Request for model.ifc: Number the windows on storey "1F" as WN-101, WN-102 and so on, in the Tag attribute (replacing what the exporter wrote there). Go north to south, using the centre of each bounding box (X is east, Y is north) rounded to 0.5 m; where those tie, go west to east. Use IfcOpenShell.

First a look at what the model holds.

```python
import ifcopenshell
import ifcopenshell.util.element
import ifcopenshell.util.placement

model = ifcopenshell.open("model.ifc")
print(model.schema)
storey = next(s for s in model.by_type("IfcBuildingStorey") if s.Name == "1F")
windows = [e for e in ifcopenshell.util.element.get_decomposition(storey) if e.is_a("IfcWindow")]
for e in sorted(windows, key=lambda e: e.id()):
    origin = ifcopenshell.util.placement.get_local_placement(e.ObjectPlacement)[:3, 3]
    print(e.id(), e.Tag, e.Name, origin.round(2) + 0.0, sep=" | ")
```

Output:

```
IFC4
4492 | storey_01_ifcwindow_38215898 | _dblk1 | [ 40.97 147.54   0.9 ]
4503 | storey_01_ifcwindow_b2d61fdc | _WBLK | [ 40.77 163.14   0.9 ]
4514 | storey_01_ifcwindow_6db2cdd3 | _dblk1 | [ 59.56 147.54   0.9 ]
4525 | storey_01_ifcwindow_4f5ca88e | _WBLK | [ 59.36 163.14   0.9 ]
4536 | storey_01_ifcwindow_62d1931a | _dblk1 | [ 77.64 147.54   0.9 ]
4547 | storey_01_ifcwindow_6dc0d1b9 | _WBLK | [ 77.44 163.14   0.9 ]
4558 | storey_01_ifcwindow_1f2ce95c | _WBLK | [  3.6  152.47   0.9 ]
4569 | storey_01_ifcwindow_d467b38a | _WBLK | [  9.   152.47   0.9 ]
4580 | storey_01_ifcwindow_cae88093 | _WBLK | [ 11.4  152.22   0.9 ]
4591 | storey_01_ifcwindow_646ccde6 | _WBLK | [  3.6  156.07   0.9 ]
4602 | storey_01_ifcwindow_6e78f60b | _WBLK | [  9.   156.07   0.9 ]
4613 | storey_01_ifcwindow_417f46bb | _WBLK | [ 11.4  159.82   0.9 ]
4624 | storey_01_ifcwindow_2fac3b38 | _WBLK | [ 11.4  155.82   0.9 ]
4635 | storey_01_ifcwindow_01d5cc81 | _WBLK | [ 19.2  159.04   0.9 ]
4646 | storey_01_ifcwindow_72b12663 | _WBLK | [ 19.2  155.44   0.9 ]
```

```python
import ifcopenshell
import ifcopenshell.geom
import ifcopenshell.util.element
import ifcopenshell.util.shape

model = ifcopenshell.open("model.ifc")
settings = ifcopenshell.geom.settings()
settings.set("use-world-coords", True)


def centre(element):
    shape = ifcopenshell.geom.create_shape(settings, element)
    return ifcopenshell.util.shape.get_bbox_centroid(shape.geometry)


storey = next(s for s in model.by_type("IfcBuildingStorey") if s.Name == "1F")
windows = [e for e in ifcopenshell.util.element.get_decomposition(storey) if e.is_a("IfcWindow")]

# Insertion points can sit at a corner or the storey origin, so sort by the geometry (in metres).
centres = {e: centre(e) for e in windows}
windows.sort(key=lambda e: (-round(centres[e][1] / 0.5), centres[e][0]))

for i, e in enumerate(windows, start=1):
    number = f"WN-1{i:02d}"
    e.Tag = number
    print(e.id(), number)

model.write("model_updated.ifc")
```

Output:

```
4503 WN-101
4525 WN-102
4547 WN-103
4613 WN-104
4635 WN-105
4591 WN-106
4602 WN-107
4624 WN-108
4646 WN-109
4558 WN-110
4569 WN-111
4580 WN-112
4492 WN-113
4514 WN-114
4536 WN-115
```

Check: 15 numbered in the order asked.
